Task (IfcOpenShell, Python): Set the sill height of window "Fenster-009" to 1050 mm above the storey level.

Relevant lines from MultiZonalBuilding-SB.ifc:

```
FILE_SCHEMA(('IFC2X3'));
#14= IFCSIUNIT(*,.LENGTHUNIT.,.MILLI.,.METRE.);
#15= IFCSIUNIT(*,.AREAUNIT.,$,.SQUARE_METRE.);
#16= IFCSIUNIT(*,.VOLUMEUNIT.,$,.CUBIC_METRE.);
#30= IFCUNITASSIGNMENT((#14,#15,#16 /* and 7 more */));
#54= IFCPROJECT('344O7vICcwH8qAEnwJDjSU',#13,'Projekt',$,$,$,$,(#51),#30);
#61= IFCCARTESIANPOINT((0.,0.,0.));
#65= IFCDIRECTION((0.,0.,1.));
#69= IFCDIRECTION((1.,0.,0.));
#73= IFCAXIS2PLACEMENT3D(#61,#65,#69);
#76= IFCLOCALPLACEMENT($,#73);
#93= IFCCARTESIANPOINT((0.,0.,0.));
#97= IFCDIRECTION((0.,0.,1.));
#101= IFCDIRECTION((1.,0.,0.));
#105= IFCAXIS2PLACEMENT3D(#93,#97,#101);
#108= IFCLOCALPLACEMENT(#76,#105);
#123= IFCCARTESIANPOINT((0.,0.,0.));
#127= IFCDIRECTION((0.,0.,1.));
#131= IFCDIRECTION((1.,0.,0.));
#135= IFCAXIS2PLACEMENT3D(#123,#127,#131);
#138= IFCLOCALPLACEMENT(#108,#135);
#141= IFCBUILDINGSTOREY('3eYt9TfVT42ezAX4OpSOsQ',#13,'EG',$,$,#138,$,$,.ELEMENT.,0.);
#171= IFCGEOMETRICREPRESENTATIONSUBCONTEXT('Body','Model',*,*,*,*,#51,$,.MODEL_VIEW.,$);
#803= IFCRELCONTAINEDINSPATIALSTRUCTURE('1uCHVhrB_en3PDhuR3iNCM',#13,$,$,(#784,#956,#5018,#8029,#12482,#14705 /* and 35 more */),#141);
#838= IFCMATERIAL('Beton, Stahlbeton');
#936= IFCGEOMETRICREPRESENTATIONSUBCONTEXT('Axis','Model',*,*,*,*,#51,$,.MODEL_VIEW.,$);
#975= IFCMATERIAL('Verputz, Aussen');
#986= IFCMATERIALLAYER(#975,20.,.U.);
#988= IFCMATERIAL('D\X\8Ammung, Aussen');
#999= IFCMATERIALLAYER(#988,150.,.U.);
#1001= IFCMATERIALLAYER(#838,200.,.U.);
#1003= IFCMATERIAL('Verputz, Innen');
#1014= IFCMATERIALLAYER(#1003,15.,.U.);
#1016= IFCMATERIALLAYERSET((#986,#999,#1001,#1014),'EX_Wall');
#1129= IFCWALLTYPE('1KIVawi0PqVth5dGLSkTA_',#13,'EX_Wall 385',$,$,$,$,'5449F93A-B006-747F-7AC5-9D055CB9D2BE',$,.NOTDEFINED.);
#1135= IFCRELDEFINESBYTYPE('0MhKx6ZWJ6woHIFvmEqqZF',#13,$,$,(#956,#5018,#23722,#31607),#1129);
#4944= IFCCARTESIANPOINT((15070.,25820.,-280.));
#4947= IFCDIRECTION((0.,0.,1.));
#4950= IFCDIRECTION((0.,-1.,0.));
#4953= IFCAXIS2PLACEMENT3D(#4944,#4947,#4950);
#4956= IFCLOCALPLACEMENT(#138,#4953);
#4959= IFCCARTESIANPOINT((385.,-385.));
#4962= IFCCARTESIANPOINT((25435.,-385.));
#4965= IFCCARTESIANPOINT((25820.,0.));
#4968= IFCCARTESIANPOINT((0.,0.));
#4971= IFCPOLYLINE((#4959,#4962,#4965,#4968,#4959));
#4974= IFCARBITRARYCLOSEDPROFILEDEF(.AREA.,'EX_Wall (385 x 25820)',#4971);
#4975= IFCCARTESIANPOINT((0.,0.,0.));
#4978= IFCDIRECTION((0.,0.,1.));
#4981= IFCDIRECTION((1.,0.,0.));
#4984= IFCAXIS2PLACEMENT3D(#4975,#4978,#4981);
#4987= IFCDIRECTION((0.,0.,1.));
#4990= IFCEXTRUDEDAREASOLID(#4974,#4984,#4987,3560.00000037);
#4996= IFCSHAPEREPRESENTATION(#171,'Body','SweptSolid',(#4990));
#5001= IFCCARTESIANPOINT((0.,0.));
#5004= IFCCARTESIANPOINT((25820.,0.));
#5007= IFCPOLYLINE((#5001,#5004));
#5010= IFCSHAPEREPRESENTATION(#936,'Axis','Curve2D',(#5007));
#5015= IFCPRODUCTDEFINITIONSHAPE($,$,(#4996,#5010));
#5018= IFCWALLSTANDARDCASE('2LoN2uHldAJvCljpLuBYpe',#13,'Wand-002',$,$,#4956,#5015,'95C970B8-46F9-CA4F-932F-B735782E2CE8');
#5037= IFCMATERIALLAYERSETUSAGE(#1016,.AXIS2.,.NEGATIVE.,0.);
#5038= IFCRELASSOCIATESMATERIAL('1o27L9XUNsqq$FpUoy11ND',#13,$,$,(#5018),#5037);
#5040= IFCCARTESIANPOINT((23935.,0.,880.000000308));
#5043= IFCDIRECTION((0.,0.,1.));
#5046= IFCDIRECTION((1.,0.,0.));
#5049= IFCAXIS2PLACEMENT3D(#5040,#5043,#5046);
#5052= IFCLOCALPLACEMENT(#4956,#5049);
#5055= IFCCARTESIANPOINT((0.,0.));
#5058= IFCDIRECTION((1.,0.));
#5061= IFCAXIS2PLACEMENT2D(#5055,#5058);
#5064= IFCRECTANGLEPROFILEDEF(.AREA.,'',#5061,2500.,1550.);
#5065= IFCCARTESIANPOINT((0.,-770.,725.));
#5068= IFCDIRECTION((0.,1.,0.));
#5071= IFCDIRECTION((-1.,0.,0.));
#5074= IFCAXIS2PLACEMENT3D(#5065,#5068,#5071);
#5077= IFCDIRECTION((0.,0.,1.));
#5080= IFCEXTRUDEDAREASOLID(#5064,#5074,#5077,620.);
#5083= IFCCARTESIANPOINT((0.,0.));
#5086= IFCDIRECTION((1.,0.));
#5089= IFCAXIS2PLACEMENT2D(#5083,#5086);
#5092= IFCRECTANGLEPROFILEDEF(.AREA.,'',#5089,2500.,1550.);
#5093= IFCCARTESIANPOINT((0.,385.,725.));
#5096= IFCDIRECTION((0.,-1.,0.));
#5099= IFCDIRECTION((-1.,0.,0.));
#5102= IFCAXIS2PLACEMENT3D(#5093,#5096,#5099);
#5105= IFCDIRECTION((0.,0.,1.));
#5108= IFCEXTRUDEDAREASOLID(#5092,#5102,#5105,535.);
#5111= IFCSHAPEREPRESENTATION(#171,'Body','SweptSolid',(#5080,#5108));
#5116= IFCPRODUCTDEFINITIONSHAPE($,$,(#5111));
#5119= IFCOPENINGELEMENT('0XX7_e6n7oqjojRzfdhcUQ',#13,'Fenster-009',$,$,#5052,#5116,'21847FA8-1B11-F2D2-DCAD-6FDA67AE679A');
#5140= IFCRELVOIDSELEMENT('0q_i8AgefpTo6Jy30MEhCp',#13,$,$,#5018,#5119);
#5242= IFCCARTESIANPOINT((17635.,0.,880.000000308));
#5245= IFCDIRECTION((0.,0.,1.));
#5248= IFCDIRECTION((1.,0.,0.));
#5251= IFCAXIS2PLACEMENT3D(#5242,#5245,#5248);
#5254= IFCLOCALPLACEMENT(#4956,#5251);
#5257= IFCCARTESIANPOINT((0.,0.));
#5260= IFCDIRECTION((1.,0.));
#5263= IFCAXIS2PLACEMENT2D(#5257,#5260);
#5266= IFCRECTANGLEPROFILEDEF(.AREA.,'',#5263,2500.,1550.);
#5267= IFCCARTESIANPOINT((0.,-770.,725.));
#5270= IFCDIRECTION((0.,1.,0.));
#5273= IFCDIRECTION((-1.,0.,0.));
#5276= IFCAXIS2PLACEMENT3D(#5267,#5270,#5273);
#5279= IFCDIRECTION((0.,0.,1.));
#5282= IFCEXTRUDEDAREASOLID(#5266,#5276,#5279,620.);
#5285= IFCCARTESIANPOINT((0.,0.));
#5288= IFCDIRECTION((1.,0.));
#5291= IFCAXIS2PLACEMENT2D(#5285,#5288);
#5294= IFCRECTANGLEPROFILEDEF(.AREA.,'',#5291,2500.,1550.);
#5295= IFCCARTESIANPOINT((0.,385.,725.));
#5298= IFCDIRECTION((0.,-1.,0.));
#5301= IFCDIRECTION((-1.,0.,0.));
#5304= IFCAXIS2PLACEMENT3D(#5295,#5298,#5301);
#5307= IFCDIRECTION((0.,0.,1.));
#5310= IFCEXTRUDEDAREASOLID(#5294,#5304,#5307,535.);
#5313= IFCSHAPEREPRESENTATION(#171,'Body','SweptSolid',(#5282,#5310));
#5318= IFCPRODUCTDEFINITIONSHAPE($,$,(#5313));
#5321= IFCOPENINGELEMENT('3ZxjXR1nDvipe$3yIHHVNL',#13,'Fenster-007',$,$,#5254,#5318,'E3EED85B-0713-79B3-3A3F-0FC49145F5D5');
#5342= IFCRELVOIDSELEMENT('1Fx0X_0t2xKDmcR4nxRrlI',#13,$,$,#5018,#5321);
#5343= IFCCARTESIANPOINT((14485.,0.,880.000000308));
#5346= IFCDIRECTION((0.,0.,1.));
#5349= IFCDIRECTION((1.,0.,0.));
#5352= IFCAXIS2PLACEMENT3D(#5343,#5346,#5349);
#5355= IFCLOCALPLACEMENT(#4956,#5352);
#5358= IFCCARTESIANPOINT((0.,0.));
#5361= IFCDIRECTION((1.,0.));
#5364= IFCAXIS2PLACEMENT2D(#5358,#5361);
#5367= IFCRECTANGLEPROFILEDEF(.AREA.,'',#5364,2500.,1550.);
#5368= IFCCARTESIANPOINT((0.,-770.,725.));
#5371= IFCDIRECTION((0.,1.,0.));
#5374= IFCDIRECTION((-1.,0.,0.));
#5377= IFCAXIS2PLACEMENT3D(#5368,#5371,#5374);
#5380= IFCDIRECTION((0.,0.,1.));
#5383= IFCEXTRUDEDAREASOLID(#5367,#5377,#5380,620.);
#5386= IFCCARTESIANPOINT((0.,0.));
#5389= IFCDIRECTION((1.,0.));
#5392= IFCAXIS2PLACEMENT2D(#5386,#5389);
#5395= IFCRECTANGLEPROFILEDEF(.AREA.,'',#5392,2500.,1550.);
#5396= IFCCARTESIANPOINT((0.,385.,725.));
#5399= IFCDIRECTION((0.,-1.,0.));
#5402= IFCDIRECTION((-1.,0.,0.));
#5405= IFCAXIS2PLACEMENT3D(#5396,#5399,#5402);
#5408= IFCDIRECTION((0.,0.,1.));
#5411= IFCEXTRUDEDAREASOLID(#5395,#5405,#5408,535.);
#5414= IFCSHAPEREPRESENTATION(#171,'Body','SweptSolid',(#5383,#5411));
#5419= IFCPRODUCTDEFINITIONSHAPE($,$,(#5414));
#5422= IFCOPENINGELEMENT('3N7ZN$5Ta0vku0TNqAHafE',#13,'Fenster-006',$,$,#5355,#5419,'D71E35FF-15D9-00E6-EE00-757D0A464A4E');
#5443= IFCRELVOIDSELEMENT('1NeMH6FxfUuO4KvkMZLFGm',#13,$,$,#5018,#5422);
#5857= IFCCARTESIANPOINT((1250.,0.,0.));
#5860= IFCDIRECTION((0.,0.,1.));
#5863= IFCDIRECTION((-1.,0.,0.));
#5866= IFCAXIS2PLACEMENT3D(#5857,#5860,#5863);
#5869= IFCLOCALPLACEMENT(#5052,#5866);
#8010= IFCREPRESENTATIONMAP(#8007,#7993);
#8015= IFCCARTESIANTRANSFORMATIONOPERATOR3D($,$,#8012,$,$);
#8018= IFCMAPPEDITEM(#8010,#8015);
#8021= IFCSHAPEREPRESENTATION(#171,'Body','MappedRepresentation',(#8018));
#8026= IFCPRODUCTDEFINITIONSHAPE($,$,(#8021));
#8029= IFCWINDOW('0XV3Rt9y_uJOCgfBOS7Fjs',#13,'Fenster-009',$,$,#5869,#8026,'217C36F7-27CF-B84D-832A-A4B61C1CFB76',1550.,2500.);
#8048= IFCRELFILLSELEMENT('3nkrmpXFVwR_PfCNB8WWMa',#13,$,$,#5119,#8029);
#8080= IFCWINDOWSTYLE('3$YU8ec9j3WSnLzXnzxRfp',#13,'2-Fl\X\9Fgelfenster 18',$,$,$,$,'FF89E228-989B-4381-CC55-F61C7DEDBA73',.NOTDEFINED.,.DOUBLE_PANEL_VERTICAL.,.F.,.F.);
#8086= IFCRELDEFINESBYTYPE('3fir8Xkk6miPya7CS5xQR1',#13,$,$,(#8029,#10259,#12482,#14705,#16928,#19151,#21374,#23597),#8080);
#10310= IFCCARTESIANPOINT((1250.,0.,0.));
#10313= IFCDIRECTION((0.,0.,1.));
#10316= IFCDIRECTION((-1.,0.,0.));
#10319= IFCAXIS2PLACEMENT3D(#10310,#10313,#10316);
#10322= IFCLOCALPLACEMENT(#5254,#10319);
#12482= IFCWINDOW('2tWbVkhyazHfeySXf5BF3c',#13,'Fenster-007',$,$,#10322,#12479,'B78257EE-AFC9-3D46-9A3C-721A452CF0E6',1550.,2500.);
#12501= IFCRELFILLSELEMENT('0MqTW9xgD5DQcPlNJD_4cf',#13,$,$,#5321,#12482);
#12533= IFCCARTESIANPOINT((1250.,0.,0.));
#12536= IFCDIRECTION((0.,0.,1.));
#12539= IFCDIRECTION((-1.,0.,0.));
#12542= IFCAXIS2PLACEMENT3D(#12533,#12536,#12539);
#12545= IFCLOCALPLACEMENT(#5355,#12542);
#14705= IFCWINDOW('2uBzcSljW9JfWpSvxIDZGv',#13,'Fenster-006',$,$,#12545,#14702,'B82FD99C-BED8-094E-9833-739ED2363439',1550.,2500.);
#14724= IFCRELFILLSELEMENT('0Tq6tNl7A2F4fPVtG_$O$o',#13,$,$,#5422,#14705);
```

```python
import numpy as np
import ifcopenshell
import ifcopenshell.api.geometry
import ifcopenshell.geom
import ifcopenshell.util.element
import ifcopenshell.util.placement
import ifcopenshell.util.shape
import ifcopenshell.util.unit

model = ifcopenshell.open("MultiZonalBuilding-SB.ifc")
unit_scale = ifcopenshell.util.unit.calculate_unit_scale(model)

window = model.by_guid("0XV3Rt9y_uJOCgfBOS7Fjs")
opening = window.FillsVoids[0].RelatingOpeningElement
storey = ifcopenshell.util.element.get_container(window, ifc_class="IfcBuildingStorey")
level = ifcopenshell.util.placement.get_local_placement(storey.ObjectPlacement)[2, 3]

# The opening's origin need not be at the sill, so measure its lowest point.
shape = ifcopenshell.geom.create_shape(ifcopenshell.geom.settings(), opening)
bottom = ifcopenshell.util.shape.get_shape_bottom_elevation(shape, shape.geometry) / unit_scale
dz = level + 1.05 / unit_scale - bottom

shift = np.array([0.0, 0.0, dz])
# The window is placed relative to its opening, so it follows when the opening moves.
matrix = ifcopenshell.util.placement.get_local_placement(opening.ObjectPlacement)
matrix[:3, 3] += shift
ifcopenshell.api.geometry.edit_object_placement(
    model, product=opening, matrix=matrix, is_si=False, should_transform_children=True
)

print(f"moved by {dz * unit_scale:+.3f} m")

model.write("MultiZonalBuilding-SB_rev.ifc")
```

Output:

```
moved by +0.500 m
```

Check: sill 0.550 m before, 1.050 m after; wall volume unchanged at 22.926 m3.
